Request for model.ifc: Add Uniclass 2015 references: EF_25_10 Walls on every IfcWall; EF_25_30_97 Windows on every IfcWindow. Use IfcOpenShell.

First a look at what the model holds.

```python
import ifcopenshell

model = ifcopenshell.open("model.ifc")
print(model.schema)
print("classifications:", [c.Name for c in model.by_type("IfcClassification")])
for ifc_class in ("IfcDoor", "IfcRoof", "IfcStair", "IfcWall", "IfcWindow"):
    print(ifc_class, len(model.by_type(ifc_class)))
```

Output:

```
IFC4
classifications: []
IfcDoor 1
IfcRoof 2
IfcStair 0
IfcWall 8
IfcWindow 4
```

```python
import ifcopenshell
import ifcopenshell.api.classification

model = ifcopenshell.open("model.ifc")

system = ifcopenshell.api.classification.add_classification(model, classification="Uniclass 2015")

codes = {
    "IfcWall": ("EF_25_10", "Walls"),
    "IfcWindow": ("EF_25_30_97", "Windows"),
}
for ifc_class, (code, name) in codes.items():
    products = model.by_type(ifc_class)
    ifcopenshell.api.classification.add_reference(
        model, products=products, classification=system, identification=code, name=name
    )
    print(code, len(products))

model.write("model_edited.ifc")
```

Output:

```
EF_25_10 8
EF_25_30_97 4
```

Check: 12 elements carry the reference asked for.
